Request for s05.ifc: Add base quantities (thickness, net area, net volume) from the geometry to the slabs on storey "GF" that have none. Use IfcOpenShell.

First a look at what the model holds.

```python
import ifcopenshell
import ifcopenshell.util.element
import ifcopenshell.util.unit

model = ifcopenshell.open("s05.ifc")
print(model.schema)
for unit_type in ("LENGTHUNIT", "AREAUNIT", "VOLUMEUNIT"):
    print(unit_type, ifcopenshell.util.unit.calculate_unit_scale(model, unit_type))
storey = next(s for s in model.by_type("IfcBuildingStorey") if s.Name == "GF")
slabs = [e for e in ifcopenshell.util.element.get_decomposition(storey) if e.is_a("IfcSlab")]
for e in sorted(slabs, key=lambda e: e.id()):
    print(e.id(), e.is_a(), e.Name, list(ifcopenshell.util.element.get_psets(e, qtos_only=True)), sep=" | ")
```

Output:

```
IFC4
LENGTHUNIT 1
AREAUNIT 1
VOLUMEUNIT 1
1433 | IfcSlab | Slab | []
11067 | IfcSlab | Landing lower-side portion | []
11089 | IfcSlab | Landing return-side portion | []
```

```python
import ifcopenshell
import ifcopenshell.api.pset
import ifcopenshell.geom
import ifcopenshell.util.element
import ifcopenshell.util.shape
import ifcopenshell.util.unit

model = ifcopenshell.open("s05.ifc")
unit_scale = ifcopenshell.util.unit.calculate_unit_scale(model)
area_scale = ifcopenshell.util.unit.calculate_unit_scale(model, "AREAUNIT")
volume_scale = ifcopenshell.util.unit.calculate_unit_scale(model, "VOLUMEUNIT")
settings = ifcopenshell.geom.settings()

storey = next(s for s in model.by_type("IfcBuildingStorey") if s.Name == "GF")
slabs = [e for e in ifcopenshell.util.element.get_decomposition(storey) if e.is_a("IfcSlab")]

for e in sorted(slabs, key=lambda e: e.id()):
    if ifcopenshell.util.element.get_psets(e, qtos_only=True, should_inherit=False):
        continue
    # Geometry comes back in metres, in the element's own axes.
    shape = ifcopenshell.geom.create_shape(settings, e)
    values = {
        "Width": ifcopenshell.util.shape.get_z(shape.geometry) / unit_scale,
        "NetArea": ifcopenshell.util.shape.get_footprint_area(shape.geometry) / area_scale,
        "NetVolume": ifcopenshell.util.shape.get_volume(shape.geometry) / volume_scale,
    }
    qto = ifcopenshell.api.pset.add_qto(model, product=e, name="Qto_SlabBaseQuantities")
    ifcopenshell.api.pset.edit_qto(model, qto=qto, properties=values)
    print(e.id(), {k: round(v, 3) for k, v in values.items()})

model.write("s05_updated.ifc")
```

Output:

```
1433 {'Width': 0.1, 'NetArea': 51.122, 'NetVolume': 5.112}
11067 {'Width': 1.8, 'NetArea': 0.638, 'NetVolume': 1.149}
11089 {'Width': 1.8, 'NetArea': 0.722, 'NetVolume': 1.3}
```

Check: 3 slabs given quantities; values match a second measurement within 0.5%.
